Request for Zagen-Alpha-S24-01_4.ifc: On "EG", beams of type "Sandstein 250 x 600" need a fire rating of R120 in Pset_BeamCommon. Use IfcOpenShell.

First a look at what the model holds.

```python
import ifcopenshell
import ifcopenshell.util.element

model = ifcopenshell.open("Zagen-Alpha-S24-01_4.ifc")
print(model.schema)
storey = next(s for s in model.by_type("IfcBuildingStorey") if s.Name == "EG")
beams = [e for e in ifcopenshell.util.element.get_decomposition(storey) if e.is_a("IfcBeam")]
seen = {}
for e in beams:
    element_type = ifcopenshell.util.element.get_type(e)
    key = (element_type.Name if element_type != e and element_type else None, ifcopenshell.util.element.get_pset(e, "Pset_BeamCommon", "FireRating"))
    seen[key] = seen.get(key, 0) + 1
for (name, value), count in sorted(seen.items(), key=str):
    print(count, "x", name, "|", value)
```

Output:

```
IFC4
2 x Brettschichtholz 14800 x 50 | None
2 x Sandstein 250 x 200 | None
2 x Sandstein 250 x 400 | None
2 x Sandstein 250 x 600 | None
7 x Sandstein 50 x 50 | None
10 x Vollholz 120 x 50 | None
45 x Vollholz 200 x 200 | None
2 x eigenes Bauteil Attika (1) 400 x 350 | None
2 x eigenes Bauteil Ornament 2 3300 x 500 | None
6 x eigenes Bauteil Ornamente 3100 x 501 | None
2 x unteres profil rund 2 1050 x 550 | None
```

```python
import ifcopenshell
import ifcopenshell.api.pset
import ifcopenshell.util.element

model = ifcopenshell.open("Zagen-Alpha-S24-01_4.ifc")

storey = next(s for s in model.by_type("IfcBuildingStorey") if s.Name == "EG")
beams = [e for e in ifcopenshell.util.element.get_decomposition(storey) if e.is_a("IfcBeam")]

count = 0
for e in beams:
    element_type = ifcopenshell.util.element.get_type(e)
    if element_type in (None, e) or element_type.Name != "Sandstein 250 x 600":
        continue
    # add_pset returns the element's existing set when there is one.
    pset = ifcopenshell.api.pset.add_pset(model, product=e, name="Pset_BeamCommon")
    ifcopenshell.api.pset.edit_pset(model, pset=pset, properties={"FireRating": "R120"})
    count += 1

print(count, "beams updated")

model.write("Zagen-Alpha-S24-01_4-out.ifc")
```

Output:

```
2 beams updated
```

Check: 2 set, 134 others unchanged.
